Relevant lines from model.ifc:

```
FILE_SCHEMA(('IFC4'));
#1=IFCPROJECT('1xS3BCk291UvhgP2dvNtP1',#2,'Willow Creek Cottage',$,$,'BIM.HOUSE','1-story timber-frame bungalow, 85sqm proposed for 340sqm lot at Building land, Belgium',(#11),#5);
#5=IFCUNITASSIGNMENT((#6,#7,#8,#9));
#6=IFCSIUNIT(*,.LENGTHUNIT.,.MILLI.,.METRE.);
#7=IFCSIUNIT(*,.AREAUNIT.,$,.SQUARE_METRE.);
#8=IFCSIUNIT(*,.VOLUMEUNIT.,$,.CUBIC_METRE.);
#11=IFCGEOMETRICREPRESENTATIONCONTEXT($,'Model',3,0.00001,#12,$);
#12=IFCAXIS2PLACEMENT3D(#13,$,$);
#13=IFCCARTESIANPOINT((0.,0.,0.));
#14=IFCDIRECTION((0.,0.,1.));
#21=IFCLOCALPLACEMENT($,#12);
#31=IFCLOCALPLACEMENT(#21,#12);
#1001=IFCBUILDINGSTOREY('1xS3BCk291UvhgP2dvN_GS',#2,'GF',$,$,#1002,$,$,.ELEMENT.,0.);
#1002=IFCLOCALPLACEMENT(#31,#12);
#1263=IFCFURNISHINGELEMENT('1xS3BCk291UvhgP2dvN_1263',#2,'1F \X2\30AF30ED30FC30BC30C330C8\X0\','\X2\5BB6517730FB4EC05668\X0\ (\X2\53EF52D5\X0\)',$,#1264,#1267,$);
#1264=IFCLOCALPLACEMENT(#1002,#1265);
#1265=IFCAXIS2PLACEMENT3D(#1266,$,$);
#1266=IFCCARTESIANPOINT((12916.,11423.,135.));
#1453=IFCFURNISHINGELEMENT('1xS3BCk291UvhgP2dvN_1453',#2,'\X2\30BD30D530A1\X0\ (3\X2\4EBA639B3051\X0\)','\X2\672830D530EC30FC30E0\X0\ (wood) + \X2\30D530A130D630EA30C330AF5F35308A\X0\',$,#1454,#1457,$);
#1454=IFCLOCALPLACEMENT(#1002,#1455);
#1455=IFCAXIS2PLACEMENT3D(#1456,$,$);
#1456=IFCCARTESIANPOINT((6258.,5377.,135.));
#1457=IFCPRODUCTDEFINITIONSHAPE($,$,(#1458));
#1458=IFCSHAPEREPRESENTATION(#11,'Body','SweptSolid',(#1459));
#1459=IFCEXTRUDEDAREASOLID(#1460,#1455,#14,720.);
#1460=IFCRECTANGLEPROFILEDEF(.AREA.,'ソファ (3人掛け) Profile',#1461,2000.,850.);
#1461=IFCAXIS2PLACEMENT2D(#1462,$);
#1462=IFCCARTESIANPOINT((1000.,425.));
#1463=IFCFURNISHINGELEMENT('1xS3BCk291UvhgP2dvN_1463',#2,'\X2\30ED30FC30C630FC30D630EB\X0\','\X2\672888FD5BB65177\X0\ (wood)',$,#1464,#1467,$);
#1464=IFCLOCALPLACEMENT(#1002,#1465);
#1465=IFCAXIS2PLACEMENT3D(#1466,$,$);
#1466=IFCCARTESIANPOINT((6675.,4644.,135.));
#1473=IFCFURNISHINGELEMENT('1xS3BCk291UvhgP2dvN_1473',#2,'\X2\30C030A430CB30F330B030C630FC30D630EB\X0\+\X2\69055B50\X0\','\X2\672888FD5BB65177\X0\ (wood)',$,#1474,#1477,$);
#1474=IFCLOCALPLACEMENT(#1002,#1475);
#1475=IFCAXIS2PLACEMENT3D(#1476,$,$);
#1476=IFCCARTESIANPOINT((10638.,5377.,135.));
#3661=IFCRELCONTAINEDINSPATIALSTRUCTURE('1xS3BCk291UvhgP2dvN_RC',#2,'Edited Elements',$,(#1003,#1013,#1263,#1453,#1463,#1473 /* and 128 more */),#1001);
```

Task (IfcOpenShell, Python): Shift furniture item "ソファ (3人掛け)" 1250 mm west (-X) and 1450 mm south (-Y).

```python
import ifcopenshell
import ifcopenshell.api.geometry
import ifcopenshell.util.placement
import ifcopenshell.util.unit

model = ifcopenshell.open("model.ifc")
unit_scale = ifcopenshell.util.unit.calculate_unit_scale(model)

item = model.by_guid("1xS3BCk291UvhgP2dvN_1453")
matrix = ifcopenshell.util.placement.get_local_placement(item.ObjectPlacement)
matrix[0, 3] -= 1.25 / unit_scale
matrix[1, 3] -= 1.45 / unit_scale
ifcopenshell.api.geometry.edit_object_placement(model, product=item, matrix=matrix, is_si=False)

print(ifcopenshell.util.placement.get_local_placement(item.ObjectPlacement).round(3) + 0.0)

model.write("model_edited.ifc")
```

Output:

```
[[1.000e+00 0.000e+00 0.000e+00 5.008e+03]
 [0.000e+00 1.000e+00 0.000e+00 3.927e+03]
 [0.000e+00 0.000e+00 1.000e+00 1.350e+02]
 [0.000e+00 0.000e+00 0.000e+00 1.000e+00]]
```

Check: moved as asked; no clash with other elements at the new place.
